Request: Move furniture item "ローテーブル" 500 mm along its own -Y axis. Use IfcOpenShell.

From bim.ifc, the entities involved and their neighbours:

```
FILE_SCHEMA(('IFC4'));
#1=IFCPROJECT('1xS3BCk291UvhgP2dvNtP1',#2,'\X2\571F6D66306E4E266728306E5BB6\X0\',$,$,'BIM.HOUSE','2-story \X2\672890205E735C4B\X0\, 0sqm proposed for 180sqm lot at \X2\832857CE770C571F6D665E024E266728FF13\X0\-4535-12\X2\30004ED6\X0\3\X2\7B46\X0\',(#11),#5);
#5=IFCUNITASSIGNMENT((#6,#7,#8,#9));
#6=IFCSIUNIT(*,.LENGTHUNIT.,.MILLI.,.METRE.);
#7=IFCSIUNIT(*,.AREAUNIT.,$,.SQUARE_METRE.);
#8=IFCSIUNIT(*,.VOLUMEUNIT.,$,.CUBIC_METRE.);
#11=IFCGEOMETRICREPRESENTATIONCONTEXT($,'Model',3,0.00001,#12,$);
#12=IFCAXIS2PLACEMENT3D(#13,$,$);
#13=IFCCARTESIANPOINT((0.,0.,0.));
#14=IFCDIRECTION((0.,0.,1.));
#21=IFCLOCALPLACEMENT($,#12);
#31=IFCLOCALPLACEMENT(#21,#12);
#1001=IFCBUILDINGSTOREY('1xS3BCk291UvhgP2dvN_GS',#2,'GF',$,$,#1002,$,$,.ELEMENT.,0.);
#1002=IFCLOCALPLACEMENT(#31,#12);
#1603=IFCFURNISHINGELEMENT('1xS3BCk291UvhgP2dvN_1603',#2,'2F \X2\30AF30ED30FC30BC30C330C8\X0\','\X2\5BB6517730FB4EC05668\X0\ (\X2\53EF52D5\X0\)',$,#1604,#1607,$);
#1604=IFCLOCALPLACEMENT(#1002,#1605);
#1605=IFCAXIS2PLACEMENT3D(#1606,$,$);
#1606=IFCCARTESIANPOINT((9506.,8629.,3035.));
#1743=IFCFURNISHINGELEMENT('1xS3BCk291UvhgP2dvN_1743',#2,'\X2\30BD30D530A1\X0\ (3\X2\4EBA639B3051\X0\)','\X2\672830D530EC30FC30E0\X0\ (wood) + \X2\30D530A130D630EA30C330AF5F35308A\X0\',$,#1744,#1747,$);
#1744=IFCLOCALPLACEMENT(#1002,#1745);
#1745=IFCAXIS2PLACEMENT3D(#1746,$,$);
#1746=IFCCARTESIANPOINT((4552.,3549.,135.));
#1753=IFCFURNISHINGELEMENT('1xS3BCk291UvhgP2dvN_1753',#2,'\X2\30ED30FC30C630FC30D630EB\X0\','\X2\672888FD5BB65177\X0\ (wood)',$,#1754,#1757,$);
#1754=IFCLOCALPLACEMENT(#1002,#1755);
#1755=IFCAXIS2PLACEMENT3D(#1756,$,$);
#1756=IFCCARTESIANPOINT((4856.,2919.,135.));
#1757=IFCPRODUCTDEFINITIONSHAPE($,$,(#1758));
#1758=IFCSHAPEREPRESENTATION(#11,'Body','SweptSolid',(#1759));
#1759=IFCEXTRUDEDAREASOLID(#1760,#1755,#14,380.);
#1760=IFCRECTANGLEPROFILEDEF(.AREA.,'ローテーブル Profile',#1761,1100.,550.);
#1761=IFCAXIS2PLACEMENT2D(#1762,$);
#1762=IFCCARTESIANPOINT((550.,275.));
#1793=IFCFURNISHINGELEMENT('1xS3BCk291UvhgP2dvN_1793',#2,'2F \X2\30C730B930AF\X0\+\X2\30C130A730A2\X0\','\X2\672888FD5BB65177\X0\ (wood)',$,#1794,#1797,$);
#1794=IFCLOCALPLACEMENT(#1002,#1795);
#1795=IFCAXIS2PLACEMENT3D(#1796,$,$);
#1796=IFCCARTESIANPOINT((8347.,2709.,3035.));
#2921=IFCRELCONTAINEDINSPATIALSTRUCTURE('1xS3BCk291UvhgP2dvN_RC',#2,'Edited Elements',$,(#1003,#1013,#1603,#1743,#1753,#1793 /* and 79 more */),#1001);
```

```python
import ifcopenshell
import ifcopenshell.api.geometry
import ifcopenshell.util.placement

model = ifcopenshell.open("bim.ifc")

item = model.by_id(1753)
matrix = ifcopenshell.util.placement.get_local_placement(item.ObjectPlacement)
matrix[:3, 3] -= matrix[:3, 1] * 500.0
ifcopenshell.api.geometry.edit_object_placement(model, product=item, matrix=matrix, is_si=False)

print(ifcopenshell.util.placement.get_local_placement(item.ObjectPlacement).round(3) + 0.0)

model.write("bim_rev.ifc")
```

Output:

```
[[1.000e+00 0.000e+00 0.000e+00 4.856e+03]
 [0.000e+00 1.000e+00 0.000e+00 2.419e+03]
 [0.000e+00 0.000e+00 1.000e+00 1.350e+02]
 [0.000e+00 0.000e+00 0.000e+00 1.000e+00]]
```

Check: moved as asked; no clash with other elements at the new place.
